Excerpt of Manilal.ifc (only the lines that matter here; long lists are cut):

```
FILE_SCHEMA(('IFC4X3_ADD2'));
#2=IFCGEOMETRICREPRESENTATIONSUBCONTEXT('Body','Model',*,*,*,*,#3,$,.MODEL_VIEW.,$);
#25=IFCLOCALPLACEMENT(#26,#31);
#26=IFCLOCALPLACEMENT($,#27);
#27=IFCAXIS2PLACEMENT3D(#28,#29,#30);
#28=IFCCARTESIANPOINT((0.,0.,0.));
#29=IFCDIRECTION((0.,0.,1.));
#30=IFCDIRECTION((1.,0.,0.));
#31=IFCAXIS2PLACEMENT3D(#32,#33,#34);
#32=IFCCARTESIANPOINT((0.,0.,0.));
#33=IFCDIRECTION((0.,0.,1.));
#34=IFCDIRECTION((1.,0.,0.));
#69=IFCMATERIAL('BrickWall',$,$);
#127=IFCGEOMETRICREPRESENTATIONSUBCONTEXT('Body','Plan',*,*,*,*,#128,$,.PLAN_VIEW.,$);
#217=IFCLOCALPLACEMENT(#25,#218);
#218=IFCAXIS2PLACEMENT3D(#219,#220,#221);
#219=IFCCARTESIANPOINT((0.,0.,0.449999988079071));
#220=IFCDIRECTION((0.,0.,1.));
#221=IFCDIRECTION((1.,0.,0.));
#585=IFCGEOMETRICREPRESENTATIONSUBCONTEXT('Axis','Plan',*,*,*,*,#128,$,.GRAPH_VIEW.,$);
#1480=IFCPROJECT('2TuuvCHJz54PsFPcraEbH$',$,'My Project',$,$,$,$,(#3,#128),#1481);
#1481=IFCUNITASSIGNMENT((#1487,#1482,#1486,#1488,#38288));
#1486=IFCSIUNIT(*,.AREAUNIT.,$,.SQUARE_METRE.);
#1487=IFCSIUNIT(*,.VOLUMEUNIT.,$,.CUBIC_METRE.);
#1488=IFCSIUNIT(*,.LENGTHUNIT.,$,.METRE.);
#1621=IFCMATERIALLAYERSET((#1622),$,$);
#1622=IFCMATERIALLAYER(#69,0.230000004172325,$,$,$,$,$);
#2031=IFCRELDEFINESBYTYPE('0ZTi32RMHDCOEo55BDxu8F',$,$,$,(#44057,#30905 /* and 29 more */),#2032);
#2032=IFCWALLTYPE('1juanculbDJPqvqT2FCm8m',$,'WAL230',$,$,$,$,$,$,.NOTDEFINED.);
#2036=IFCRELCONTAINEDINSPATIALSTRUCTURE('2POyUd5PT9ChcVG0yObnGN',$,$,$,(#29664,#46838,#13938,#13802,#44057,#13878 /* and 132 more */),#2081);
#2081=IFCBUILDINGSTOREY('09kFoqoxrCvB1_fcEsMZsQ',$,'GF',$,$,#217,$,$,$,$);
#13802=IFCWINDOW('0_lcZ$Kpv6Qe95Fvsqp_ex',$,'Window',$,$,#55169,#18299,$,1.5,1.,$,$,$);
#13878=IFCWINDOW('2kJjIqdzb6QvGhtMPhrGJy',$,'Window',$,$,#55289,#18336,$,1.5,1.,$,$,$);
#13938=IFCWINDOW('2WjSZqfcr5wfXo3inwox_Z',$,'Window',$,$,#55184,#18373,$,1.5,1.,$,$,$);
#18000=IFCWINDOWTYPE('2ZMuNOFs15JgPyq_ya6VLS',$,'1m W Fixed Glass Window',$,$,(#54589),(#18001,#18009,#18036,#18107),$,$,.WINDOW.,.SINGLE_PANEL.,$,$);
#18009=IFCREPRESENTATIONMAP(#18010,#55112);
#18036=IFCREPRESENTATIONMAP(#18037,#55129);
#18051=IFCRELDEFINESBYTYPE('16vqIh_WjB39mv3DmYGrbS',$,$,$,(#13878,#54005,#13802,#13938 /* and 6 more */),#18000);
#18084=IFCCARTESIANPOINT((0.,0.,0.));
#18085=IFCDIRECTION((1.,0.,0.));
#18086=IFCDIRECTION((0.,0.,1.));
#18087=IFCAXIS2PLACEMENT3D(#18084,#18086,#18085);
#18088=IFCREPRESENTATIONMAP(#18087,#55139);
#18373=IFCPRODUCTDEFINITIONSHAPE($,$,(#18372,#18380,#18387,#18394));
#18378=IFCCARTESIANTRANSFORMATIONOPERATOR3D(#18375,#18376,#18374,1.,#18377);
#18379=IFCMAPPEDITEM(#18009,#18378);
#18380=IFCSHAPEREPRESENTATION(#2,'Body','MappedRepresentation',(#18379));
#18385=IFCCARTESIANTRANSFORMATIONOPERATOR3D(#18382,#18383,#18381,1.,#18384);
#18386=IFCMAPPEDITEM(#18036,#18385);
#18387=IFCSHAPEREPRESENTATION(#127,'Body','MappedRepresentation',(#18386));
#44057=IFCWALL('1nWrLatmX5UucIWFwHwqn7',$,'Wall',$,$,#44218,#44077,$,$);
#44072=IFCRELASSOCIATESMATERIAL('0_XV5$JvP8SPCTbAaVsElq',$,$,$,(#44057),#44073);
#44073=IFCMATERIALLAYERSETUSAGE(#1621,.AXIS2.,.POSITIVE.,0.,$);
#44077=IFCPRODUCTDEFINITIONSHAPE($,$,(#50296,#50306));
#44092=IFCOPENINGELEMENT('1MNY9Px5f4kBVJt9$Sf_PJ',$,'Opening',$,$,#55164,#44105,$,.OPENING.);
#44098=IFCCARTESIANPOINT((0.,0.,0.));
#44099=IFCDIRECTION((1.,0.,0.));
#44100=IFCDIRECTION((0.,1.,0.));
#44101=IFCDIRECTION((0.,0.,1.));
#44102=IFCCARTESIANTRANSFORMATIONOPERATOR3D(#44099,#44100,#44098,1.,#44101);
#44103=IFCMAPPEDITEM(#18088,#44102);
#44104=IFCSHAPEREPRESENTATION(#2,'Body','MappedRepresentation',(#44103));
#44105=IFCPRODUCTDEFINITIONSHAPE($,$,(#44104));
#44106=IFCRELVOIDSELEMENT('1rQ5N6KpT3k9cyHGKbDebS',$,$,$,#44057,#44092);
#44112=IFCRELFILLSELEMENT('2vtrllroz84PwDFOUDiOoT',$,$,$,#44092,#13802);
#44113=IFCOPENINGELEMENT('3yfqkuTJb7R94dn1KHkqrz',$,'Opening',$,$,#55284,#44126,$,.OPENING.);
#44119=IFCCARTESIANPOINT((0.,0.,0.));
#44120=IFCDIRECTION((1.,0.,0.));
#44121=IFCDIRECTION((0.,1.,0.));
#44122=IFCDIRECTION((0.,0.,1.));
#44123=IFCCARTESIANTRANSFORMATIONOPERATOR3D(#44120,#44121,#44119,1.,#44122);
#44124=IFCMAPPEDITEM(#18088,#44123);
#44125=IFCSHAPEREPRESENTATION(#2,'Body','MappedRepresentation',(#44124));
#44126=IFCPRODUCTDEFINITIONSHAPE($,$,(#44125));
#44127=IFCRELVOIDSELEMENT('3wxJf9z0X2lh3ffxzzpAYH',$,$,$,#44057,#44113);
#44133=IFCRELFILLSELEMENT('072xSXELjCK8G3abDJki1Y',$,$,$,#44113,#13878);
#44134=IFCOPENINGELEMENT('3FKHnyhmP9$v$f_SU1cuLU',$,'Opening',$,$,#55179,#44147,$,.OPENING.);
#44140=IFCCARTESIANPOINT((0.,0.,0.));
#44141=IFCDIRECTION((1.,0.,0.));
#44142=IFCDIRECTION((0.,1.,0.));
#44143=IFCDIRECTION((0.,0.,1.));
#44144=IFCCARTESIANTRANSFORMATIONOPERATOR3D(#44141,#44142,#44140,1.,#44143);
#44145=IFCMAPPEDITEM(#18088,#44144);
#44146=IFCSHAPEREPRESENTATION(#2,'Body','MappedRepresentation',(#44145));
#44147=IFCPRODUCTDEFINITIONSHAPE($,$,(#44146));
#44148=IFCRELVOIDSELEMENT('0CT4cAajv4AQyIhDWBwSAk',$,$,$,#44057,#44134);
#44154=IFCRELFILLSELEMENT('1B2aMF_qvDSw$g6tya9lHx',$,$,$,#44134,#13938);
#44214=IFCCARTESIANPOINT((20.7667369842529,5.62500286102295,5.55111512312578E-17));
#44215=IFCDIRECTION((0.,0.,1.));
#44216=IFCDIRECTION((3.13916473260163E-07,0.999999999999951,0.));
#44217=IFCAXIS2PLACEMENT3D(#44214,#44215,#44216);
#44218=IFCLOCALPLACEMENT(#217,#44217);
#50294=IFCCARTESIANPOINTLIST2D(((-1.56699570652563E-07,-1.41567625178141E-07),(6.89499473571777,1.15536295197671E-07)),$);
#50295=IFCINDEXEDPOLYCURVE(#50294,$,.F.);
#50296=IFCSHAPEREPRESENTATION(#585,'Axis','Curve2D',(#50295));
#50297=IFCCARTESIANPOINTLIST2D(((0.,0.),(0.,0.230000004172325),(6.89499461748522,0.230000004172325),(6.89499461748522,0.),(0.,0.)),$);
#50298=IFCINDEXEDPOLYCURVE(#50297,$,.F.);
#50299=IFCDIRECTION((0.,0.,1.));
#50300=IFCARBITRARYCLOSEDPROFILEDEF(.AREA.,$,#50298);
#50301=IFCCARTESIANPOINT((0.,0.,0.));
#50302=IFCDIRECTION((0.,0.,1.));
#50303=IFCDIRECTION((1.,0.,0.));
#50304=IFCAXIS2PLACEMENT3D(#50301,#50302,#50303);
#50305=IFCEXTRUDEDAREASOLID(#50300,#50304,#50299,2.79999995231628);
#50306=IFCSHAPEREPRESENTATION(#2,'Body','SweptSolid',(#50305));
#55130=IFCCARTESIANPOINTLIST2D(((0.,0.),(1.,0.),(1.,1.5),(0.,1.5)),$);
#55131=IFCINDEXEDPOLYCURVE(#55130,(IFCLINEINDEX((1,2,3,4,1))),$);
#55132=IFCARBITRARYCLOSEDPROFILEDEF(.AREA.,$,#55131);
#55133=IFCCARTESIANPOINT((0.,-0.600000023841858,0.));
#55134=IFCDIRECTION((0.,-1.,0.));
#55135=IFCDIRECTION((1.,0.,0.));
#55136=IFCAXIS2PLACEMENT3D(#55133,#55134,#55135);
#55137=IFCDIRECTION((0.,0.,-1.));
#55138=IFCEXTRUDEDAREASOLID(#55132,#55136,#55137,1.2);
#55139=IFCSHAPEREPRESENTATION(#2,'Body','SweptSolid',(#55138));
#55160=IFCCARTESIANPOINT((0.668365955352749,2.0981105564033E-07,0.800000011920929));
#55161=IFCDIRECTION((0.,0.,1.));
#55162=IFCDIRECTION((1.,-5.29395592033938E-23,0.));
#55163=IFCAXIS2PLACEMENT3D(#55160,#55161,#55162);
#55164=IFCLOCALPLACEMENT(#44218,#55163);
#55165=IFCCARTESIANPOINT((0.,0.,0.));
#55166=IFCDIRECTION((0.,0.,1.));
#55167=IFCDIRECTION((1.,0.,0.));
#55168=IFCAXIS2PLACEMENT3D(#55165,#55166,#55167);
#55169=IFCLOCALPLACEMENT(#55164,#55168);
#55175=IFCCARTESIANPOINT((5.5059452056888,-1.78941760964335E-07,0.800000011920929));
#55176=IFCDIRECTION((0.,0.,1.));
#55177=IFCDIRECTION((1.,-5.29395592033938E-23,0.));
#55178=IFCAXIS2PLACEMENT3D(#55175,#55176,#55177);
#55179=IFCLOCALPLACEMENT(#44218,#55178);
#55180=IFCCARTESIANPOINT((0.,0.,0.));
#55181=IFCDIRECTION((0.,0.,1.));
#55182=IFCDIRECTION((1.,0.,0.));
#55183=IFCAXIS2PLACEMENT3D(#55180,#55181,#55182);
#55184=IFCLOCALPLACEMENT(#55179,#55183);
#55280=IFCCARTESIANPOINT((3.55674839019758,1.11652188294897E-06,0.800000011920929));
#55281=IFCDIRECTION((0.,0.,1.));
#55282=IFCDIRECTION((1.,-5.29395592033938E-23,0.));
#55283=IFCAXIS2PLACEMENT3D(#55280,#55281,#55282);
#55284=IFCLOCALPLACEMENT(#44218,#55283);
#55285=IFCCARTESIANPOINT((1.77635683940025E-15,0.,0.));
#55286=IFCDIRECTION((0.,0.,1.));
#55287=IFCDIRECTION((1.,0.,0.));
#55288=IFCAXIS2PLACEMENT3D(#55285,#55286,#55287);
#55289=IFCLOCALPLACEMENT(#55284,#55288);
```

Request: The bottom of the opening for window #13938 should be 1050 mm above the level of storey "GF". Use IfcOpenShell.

```python
import numpy as np
import ifcopenshell
import ifcopenshell.api.geometry
import ifcopenshell.geom
import ifcopenshell.util.element
import ifcopenshell.util.placement
import ifcopenshell.util.shape
import ifcopenshell.util.unit

model = ifcopenshell.open("Manilal.ifc")
unit_scale = ifcopenshell.util.unit.calculate_unit_scale(model)

window = model.by_guid("2WjSZqfcr5wfXo3inwox_Z")
opening = window.FillsVoids[0].RelatingOpeningElement
storey = ifcopenshell.util.element.get_container(window, ifc_class="IfcBuildingStorey")
level = ifcopenshell.util.placement.get_local_placement(storey.ObjectPlacement)[2, 3]

# The opening's origin need not be at the sill, so measure its lowest point.
shape = ifcopenshell.geom.create_shape(ifcopenshell.geom.settings(), opening)
bottom = ifcopenshell.util.shape.get_shape_bottom_elevation(shape, shape.geometry) / unit_scale
dz = level + 1.05 / unit_scale - bottom

shift = np.array([0.0, 0.0, dz])
# The window is placed relative to its opening, so it follows when the opening moves.
matrix = ifcopenshell.util.placement.get_local_placement(opening.ObjectPlacement)
matrix[:3, 3] += shift
ifcopenshell.api.geometry.edit_object_placement(
    model, product=opening, matrix=matrix, is_si=False, should_transform_children=True
)

print(f"moved by {dz * unit_scale:+.3f} m")

model.write("Manilal_v2.ifc")
```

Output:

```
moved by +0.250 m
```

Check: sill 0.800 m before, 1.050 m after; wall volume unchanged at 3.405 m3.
